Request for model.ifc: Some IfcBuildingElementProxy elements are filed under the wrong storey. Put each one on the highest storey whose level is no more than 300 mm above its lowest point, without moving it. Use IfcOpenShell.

First a look at what the model holds.

```python
import ifcopenshell
import ifcopenshell.util.element
import ifcopenshell.util.placement

model = ifcopenshell.open("model.ifc")
print(model.schema)
for storey in model.by_type("IfcBuildingStorey"):
    level = ifcopenshell.util.placement.get_storey_elevation(storey)
    count = sum(e.is_a("IfcBuildingElementProxy") for e in ifcopenshell.util.element.get_contained(storey))
    print(storey.id(), storey.Name, round(level, 3), count, sep=" | ")
```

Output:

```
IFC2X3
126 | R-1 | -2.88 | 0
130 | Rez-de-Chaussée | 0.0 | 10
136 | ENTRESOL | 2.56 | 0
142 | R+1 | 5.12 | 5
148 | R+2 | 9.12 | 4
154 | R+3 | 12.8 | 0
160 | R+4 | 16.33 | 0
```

```python
import ifcopenshell
import ifcopenshell.api.spatial
import ifcopenshell.geom
import ifcopenshell.util.element
import ifcopenshell.util.placement
import ifcopenshell.util.shape
import ifcopenshell.util.unit

model = ifcopenshell.open("model.ifc")
unit_scale = ifcopenshell.util.unit.calculate_unit_scale(model)
settings = ifcopenshell.geom.settings()

levels = sorted(
    ((ifcopenshell.util.placement.get_storey_elevation(s) * unit_scale, s) for s in model.by_type("IfcBuildingStorey")),
    key=lambda pair: pair[0],
)

for e in model.by_type("IfcBuildingElementProxy"):
    current = e.ContainedInStructure[0].RelatingStructure if e.ContainedInStructure else None
    if current is None or not current.is_a("IfcBuildingStorey"):
        continue
    shape = ifcopenshell.geom.create_shape(settings, e)
    bottom = ifcopenshell.util.shape.get_shape_bottom_elevation(shape, shape.geometry)
    below = [s for level, s in levels if level <= bottom + 0.3]
    storey = below[-1] if below else levels[0][1]
    if storey != current:
        # assign_container keeps the world position.
        ifcopenshell.api.spatial.assign_container(model, products=[e], relating_structure=storey)
        print(e.id(), current.Name, "->", storey.Name)

model.write("model_v2.ifc")
```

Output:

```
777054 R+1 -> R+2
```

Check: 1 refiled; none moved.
